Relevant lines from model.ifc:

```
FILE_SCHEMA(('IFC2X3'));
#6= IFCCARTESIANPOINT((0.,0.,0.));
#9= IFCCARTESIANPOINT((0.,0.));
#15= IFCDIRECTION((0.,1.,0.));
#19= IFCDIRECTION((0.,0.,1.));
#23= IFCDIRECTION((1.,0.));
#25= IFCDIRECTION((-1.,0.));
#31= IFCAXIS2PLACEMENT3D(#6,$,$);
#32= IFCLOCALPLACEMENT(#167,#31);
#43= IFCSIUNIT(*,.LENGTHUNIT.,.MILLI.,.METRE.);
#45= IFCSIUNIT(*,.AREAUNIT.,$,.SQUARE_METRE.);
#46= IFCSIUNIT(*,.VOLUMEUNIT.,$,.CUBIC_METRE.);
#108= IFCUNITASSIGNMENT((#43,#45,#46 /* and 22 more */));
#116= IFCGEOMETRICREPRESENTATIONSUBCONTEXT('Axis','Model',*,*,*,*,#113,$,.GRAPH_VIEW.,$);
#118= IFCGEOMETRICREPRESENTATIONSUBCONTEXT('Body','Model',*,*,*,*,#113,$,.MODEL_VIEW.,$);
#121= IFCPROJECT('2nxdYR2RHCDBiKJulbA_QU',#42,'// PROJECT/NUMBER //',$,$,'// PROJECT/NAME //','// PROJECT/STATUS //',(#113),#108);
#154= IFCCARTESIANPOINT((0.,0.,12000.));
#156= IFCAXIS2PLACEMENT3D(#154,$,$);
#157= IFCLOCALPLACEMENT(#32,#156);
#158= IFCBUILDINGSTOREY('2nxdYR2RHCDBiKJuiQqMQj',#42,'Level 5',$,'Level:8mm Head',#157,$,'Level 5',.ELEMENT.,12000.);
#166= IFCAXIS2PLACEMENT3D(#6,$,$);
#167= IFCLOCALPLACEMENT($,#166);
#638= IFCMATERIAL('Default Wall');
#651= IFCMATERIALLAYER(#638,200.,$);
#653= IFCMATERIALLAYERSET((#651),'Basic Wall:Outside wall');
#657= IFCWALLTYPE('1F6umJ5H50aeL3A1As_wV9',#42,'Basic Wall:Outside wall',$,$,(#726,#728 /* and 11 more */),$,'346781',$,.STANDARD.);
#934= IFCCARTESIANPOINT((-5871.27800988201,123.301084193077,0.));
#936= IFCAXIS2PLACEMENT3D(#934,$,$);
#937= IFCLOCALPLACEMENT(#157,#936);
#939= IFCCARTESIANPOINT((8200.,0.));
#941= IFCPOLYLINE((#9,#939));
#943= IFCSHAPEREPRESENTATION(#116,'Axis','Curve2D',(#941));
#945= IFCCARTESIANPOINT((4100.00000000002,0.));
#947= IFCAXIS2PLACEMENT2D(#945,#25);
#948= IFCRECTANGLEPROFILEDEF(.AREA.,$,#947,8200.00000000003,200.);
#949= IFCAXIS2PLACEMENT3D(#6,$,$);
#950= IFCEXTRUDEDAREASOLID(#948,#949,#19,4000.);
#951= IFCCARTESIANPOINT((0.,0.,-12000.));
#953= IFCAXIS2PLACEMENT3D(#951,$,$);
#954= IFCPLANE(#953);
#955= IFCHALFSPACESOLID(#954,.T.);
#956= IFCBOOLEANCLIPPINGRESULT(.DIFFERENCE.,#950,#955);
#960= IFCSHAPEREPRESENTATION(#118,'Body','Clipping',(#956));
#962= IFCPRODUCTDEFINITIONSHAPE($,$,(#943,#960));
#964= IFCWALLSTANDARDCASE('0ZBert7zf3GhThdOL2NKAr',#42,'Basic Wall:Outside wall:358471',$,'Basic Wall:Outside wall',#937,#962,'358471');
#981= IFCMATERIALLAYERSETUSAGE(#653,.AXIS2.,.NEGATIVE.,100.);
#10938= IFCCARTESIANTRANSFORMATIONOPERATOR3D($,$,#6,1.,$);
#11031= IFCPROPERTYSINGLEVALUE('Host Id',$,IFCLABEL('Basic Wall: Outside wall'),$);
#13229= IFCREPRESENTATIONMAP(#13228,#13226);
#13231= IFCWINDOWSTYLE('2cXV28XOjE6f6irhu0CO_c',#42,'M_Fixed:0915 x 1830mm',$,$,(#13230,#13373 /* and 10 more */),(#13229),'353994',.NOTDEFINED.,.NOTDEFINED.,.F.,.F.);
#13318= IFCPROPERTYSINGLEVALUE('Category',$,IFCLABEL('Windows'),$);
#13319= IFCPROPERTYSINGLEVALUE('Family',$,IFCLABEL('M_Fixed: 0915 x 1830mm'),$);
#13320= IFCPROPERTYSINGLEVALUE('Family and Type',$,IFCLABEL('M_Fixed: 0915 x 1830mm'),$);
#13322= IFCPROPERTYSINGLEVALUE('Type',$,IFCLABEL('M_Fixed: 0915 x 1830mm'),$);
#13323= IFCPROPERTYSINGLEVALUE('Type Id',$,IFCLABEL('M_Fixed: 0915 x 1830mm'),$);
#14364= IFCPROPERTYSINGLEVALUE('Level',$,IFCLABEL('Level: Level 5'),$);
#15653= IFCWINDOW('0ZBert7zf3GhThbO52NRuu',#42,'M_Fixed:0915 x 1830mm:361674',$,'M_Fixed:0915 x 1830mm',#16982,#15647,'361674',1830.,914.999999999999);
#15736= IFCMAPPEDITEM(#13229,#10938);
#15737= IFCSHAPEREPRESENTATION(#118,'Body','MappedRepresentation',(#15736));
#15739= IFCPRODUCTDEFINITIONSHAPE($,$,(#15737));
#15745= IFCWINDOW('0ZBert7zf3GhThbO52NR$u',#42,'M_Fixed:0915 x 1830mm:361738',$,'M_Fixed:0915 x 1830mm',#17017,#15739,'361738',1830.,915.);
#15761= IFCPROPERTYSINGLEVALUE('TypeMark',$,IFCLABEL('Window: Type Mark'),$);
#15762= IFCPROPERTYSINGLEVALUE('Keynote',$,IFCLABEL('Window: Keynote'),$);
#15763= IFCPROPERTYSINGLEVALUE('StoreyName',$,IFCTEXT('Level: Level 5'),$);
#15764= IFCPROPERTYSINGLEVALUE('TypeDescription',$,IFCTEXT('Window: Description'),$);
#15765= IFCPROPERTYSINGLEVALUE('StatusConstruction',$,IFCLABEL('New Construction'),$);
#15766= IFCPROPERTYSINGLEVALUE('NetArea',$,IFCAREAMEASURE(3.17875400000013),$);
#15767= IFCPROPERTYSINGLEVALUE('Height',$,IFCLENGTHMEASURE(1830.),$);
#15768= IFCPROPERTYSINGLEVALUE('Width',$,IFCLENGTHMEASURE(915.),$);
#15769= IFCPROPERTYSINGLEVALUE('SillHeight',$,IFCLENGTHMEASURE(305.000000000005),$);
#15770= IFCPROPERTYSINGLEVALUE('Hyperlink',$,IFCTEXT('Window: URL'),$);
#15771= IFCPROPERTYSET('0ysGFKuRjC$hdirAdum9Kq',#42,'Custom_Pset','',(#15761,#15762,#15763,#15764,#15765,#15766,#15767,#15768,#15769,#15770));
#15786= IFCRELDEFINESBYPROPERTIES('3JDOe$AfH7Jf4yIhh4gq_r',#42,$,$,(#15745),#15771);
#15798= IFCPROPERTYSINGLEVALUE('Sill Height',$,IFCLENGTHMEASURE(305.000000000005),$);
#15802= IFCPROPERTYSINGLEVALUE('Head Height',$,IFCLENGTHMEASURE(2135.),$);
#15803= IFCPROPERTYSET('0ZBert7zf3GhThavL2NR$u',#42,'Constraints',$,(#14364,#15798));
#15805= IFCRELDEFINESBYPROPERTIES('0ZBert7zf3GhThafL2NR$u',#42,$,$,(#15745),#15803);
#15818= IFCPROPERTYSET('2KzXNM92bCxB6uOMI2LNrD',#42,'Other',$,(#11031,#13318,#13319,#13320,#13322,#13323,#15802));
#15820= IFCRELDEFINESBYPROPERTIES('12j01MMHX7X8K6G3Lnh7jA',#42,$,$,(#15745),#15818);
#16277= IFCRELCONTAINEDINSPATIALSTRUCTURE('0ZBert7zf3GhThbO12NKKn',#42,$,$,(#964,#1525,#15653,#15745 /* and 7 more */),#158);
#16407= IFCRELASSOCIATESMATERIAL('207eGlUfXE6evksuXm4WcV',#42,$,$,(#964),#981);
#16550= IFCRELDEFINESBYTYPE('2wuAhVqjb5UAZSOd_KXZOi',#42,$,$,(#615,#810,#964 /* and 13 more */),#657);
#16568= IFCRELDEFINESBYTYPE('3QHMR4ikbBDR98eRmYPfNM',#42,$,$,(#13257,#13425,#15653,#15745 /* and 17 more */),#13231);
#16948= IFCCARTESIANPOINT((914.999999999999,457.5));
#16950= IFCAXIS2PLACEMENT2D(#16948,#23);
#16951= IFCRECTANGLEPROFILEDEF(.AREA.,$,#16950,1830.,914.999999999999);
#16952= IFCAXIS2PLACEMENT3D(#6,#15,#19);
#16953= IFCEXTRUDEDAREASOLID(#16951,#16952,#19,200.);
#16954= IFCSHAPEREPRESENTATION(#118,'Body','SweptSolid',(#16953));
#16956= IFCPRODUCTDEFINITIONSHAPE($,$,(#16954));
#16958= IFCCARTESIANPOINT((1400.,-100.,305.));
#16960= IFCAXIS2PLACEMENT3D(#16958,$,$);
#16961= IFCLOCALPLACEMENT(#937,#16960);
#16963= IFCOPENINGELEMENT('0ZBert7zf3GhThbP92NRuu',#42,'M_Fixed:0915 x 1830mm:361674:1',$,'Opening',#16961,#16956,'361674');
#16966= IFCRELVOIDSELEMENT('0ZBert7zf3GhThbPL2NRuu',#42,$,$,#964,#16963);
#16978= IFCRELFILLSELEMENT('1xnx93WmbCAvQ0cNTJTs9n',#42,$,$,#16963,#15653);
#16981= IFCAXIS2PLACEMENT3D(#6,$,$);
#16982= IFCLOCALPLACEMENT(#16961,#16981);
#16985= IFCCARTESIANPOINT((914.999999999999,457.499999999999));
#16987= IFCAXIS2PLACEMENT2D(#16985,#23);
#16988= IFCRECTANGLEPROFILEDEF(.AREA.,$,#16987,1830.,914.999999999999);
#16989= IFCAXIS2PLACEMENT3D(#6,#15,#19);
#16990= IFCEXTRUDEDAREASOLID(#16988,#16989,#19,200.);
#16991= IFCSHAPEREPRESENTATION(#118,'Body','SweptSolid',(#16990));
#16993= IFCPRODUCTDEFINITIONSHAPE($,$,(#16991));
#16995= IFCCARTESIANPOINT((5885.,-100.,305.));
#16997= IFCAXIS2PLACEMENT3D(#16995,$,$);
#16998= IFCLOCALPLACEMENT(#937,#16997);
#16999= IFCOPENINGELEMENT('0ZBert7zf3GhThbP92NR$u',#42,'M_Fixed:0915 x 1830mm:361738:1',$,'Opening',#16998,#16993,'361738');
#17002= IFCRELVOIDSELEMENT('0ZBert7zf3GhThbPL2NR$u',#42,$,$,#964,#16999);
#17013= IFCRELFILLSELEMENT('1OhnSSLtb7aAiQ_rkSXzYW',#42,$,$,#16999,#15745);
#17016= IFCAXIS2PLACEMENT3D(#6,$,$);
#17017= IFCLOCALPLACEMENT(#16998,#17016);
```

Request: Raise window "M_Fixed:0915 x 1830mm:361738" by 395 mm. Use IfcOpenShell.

```python
import numpy as np
import ifcopenshell
import ifcopenshell.api.geometry
import ifcopenshell.api.pset
import ifcopenshell.util.element
import ifcopenshell.util.placement
import ifcopenshell.util.unit

model = ifcopenshell.open("model.ifc")
unit_scale = ifcopenshell.util.unit.calculate_unit_scale(model)

window = model.by_id(15745)
opening = window.FillsVoids[0].RelatingOpeningElement
dz = 0.395 / unit_scale

shift = np.array([0.0, 0.0, dz])
# The window is placed relative to its opening, so it follows when the opening moves.
matrix = ifcopenshell.util.placement.get_local_placement(opening.ObjectPlacement)
matrix[:3, 3] += shift
ifcopenshell.api.geometry.edit_object_placement(
    model, product=opening, matrix=matrix, is_si=False, should_transform_children=True
)

# Keep the stored heights in step.
pset = model.by_id(ifcopenshell.util.element.get_pset(window, "Custom_Pset", should_inherit=False)["id"])
ifcopenshell.api.pset.edit_pset(model, pset=pset, properties={
    "SillHeight": model.create_entity("IfcLengthMeasure", ifcopenshell.util.element.get_pset(window, "Constraints", "Sill Height") + dz),
})
pset = model.by_id(ifcopenshell.util.element.get_pset(window, "Constraints", should_inherit=False)["id"])
ifcopenshell.api.pset.edit_pset(model, pset=pset, properties={
    "Sill Height": model.create_entity("IfcLengthMeasure", ifcopenshell.util.element.get_pset(window, "Constraints", "Sill Height") + dz),
})
pset = model.by_id(ifcopenshell.util.element.get_pset(window, "Other", should_inherit=False)["id"])
ifcopenshell.api.pset.edit_pset(model, pset=pset, properties={
    "Head Height": model.create_entity("IfcLengthMeasure", ifcopenshell.util.element.get_pset(window, "Other", "Head Height") + dz),
})

print(f"moved by {dz * unit_scale:+.3f} m")

model.write("model_edited.ifc")
```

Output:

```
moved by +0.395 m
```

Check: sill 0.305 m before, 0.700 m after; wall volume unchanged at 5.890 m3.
